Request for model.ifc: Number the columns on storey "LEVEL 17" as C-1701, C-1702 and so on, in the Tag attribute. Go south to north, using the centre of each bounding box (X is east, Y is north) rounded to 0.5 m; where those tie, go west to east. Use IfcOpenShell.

First a look at what the model holds.

```python
import ifcopenshell
import ifcopenshell.util.element
import ifcopenshell.util.placement

model = ifcopenshell.open("model.ifc")
print(model.schema)
storey = next(s for s in model.by_type("IfcBuildingStorey") if s.Name == "LEVEL 17")
columns = [e for e in ifcopenshell.util.element.get_decomposition(storey) if e.is_a("IfcColumn")]
for e in sorted(columns, key=lambda e: e.id()):
    origin = ifcopenshell.util.placement.get_local_placement(e.ObjectPlacement)[:3, 3]
    print(e.id(), e.Tag, e.Name, origin.round(2) + 0.0, sep=" | ")
```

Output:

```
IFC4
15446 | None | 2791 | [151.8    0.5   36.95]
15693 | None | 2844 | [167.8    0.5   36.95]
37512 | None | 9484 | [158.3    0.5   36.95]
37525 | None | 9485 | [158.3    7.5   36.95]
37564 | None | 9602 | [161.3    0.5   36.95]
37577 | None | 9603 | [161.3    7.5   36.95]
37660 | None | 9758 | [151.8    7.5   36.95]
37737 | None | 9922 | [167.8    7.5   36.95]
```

```python
import ifcopenshell
import ifcopenshell.geom
import ifcopenshell.util.element
import ifcopenshell.util.shape

model = ifcopenshell.open("model.ifc")
settings = ifcopenshell.geom.settings()
settings.set("use-world-coords", True)


def centre(element):
    shape = ifcopenshell.geom.create_shape(settings, element)
    return ifcopenshell.util.shape.get_bbox_centroid(shape.geometry)


storey = next(s for s in model.by_type("IfcBuildingStorey") if s.Name == "LEVEL 17")
columns = [e for e in ifcopenshell.util.element.get_decomposition(storey) if e.is_a("IfcColumn")]

# Insertion points can sit at a corner or the storey origin, so sort by the geometry (in metres).
centres = {e: centre(e) for e in columns}
columns.sort(key=lambda e: (round(centres[e][1] / 0.5), centres[e][0]))

for i, e in enumerate(columns, start=1):
    number = f"C-17{i:02d}"
    e.Tag = number
    print(e.id(), number)

model.write("model-out.ifc")
```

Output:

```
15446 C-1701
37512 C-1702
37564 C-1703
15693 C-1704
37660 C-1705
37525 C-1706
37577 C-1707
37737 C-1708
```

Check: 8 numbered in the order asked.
